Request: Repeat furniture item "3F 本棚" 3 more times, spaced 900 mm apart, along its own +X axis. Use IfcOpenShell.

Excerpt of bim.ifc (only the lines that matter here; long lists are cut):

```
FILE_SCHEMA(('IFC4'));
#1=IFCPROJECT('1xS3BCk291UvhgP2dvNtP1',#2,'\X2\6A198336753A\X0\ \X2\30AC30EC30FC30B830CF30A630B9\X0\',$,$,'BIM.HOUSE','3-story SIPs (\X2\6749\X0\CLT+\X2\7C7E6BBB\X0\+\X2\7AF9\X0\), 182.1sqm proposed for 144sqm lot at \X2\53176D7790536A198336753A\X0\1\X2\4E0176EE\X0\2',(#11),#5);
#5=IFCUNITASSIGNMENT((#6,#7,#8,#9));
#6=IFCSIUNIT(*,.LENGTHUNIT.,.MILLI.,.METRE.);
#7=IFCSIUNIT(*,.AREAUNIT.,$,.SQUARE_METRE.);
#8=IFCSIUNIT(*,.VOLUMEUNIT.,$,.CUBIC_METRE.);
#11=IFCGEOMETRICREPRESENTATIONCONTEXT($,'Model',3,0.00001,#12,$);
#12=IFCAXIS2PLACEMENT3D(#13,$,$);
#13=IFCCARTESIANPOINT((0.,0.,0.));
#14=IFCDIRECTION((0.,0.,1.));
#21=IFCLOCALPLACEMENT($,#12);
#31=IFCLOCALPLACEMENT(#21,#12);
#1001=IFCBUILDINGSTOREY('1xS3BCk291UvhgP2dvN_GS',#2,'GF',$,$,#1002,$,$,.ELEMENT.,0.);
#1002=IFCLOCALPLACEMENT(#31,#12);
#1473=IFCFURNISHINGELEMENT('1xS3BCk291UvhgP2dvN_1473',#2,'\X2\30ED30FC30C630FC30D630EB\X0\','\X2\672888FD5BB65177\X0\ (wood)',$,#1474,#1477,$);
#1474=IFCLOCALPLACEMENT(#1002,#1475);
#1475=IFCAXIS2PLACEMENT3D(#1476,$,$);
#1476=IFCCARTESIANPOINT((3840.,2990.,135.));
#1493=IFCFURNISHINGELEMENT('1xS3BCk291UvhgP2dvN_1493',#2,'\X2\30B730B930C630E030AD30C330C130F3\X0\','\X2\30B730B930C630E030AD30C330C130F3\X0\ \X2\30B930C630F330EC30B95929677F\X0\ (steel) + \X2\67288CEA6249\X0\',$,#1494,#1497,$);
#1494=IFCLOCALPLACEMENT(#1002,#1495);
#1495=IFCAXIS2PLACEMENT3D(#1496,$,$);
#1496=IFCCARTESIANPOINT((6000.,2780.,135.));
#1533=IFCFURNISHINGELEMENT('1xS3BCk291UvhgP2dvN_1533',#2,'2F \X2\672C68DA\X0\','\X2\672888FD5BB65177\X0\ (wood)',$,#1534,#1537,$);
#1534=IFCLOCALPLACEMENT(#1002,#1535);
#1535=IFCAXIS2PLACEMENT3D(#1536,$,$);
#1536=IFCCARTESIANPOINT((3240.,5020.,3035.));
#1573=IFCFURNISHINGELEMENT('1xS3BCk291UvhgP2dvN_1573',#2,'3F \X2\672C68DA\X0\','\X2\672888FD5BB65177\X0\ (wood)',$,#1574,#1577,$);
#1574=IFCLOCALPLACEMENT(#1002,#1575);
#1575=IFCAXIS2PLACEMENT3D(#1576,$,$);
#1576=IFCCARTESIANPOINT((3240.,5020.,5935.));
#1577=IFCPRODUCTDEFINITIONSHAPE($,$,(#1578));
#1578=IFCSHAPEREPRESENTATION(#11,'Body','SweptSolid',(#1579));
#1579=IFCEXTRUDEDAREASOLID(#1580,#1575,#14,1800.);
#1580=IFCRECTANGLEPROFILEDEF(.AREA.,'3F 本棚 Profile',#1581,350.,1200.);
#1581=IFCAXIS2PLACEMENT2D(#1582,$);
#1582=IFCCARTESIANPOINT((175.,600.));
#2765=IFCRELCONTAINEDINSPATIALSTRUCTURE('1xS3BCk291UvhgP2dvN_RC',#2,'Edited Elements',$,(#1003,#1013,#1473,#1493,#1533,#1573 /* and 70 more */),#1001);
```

```python
import ifcopenshell
import ifcopenshell.api.geometry
import ifcopenshell.api.root
import ifcopenshell.util.element
import ifcopenshell.util.placement

model = ifcopenshell.open("bim.ifc")


def reuse_history(source, copy):
    """copy_class also copies each property set's owner history, people and application; keep the originals."""
    for rel in copy.IsDefinedBy:
        if rel.is_a("IfcRelDefinesByProperties") and (history := rel.RelatingPropertyDefinition.OwnerHistory):
            rel.RelatingPropertyDefinition.OwnerHistory = source.OwnerHistory
            ifcopenshell.util.element.remove_deep2(model, history)


source = model.by_id(1573)
base = ifcopenshell.util.placement.get_local_placement(source.ObjectPlacement)
step = base[:3, 0] * 900.0

for i in range(1, 4):
    copy = ifcopenshell.api.root.copy_class(model, product=source)
    copy.Representation = ifcopenshell.util.element.copy_deep(
        model, source.Representation, exclude=["IfcGeometricRepresentationContext", "IfcRepresentationMap"]
    )
    reuse_history(source, copy)
    matrix = base.copy()
    matrix[:3, 3] += i * step
    print("added at", matrix[:3, 3].round(3) + 0.0)
    ifcopenshell.api.geometry.edit_object_placement(model, product=copy, matrix=matrix, is_si=False)

model.write("bim_rev.ifc")
```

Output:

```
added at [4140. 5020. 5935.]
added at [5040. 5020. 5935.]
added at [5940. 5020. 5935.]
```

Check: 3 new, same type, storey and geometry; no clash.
